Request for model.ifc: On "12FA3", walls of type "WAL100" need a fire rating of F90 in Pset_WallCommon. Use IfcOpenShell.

First a look at what the model holds.

```python
import ifcopenshell
import ifcopenshell.util.element

model = ifcopenshell.open("model.ifc")
print(model.schema)
storey = next(s for s in model.by_type("IfcBuildingStorey") if s.Name == "12FA3")
walls = [e for e in ifcopenshell.util.element.get_decomposition(storey) if e.is_a("IfcWall")]
seen = {}
for e in walls:
    element_type = ifcopenshell.util.element.get_type(e)
    key = (element_type.Name if element_type != e and element_type else None, ifcopenshell.util.element.get_pset(e, "Pset_WallCommon", "FireRating"))
    seen[key] = seen.get(key, 0) + 1
for (name, value), count in sorted(seen.items(), key=str):
    print(count, "x", name, "|", value)
```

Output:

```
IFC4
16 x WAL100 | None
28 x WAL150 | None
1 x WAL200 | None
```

```python
import ifcopenshell
import ifcopenshell.api.pset
import ifcopenshell.util.element

model = ifcopenshell.open("model.ifc")

storey = next(s for s in model.by_type("IfcBuildingStorey") if s.Name == "12FA3")
walls = [e for e in ifcopenshell.util.element.get_decomposition(storey) if e.is_a("IfcWall")]

count = 0
for e in walls:
    element_type = ifcopenshell.util.element.get_type(e)
    if element_type in (None, e) or element_type.Name != "WAL100":
        continue
    # add_pset returns the element's existing set when there is one.
    pset = ifcopenshell.api.pset.add_pset(model, product=e, name="Pset_WallCommon")
    ifcopenshell.api.pset.edit_pset(model, pset=pset, properties={"FireRating": "F90"})
    count += 1

print(count, "walls updated")

model.write("model-out.ifc")
```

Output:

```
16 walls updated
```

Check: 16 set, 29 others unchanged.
